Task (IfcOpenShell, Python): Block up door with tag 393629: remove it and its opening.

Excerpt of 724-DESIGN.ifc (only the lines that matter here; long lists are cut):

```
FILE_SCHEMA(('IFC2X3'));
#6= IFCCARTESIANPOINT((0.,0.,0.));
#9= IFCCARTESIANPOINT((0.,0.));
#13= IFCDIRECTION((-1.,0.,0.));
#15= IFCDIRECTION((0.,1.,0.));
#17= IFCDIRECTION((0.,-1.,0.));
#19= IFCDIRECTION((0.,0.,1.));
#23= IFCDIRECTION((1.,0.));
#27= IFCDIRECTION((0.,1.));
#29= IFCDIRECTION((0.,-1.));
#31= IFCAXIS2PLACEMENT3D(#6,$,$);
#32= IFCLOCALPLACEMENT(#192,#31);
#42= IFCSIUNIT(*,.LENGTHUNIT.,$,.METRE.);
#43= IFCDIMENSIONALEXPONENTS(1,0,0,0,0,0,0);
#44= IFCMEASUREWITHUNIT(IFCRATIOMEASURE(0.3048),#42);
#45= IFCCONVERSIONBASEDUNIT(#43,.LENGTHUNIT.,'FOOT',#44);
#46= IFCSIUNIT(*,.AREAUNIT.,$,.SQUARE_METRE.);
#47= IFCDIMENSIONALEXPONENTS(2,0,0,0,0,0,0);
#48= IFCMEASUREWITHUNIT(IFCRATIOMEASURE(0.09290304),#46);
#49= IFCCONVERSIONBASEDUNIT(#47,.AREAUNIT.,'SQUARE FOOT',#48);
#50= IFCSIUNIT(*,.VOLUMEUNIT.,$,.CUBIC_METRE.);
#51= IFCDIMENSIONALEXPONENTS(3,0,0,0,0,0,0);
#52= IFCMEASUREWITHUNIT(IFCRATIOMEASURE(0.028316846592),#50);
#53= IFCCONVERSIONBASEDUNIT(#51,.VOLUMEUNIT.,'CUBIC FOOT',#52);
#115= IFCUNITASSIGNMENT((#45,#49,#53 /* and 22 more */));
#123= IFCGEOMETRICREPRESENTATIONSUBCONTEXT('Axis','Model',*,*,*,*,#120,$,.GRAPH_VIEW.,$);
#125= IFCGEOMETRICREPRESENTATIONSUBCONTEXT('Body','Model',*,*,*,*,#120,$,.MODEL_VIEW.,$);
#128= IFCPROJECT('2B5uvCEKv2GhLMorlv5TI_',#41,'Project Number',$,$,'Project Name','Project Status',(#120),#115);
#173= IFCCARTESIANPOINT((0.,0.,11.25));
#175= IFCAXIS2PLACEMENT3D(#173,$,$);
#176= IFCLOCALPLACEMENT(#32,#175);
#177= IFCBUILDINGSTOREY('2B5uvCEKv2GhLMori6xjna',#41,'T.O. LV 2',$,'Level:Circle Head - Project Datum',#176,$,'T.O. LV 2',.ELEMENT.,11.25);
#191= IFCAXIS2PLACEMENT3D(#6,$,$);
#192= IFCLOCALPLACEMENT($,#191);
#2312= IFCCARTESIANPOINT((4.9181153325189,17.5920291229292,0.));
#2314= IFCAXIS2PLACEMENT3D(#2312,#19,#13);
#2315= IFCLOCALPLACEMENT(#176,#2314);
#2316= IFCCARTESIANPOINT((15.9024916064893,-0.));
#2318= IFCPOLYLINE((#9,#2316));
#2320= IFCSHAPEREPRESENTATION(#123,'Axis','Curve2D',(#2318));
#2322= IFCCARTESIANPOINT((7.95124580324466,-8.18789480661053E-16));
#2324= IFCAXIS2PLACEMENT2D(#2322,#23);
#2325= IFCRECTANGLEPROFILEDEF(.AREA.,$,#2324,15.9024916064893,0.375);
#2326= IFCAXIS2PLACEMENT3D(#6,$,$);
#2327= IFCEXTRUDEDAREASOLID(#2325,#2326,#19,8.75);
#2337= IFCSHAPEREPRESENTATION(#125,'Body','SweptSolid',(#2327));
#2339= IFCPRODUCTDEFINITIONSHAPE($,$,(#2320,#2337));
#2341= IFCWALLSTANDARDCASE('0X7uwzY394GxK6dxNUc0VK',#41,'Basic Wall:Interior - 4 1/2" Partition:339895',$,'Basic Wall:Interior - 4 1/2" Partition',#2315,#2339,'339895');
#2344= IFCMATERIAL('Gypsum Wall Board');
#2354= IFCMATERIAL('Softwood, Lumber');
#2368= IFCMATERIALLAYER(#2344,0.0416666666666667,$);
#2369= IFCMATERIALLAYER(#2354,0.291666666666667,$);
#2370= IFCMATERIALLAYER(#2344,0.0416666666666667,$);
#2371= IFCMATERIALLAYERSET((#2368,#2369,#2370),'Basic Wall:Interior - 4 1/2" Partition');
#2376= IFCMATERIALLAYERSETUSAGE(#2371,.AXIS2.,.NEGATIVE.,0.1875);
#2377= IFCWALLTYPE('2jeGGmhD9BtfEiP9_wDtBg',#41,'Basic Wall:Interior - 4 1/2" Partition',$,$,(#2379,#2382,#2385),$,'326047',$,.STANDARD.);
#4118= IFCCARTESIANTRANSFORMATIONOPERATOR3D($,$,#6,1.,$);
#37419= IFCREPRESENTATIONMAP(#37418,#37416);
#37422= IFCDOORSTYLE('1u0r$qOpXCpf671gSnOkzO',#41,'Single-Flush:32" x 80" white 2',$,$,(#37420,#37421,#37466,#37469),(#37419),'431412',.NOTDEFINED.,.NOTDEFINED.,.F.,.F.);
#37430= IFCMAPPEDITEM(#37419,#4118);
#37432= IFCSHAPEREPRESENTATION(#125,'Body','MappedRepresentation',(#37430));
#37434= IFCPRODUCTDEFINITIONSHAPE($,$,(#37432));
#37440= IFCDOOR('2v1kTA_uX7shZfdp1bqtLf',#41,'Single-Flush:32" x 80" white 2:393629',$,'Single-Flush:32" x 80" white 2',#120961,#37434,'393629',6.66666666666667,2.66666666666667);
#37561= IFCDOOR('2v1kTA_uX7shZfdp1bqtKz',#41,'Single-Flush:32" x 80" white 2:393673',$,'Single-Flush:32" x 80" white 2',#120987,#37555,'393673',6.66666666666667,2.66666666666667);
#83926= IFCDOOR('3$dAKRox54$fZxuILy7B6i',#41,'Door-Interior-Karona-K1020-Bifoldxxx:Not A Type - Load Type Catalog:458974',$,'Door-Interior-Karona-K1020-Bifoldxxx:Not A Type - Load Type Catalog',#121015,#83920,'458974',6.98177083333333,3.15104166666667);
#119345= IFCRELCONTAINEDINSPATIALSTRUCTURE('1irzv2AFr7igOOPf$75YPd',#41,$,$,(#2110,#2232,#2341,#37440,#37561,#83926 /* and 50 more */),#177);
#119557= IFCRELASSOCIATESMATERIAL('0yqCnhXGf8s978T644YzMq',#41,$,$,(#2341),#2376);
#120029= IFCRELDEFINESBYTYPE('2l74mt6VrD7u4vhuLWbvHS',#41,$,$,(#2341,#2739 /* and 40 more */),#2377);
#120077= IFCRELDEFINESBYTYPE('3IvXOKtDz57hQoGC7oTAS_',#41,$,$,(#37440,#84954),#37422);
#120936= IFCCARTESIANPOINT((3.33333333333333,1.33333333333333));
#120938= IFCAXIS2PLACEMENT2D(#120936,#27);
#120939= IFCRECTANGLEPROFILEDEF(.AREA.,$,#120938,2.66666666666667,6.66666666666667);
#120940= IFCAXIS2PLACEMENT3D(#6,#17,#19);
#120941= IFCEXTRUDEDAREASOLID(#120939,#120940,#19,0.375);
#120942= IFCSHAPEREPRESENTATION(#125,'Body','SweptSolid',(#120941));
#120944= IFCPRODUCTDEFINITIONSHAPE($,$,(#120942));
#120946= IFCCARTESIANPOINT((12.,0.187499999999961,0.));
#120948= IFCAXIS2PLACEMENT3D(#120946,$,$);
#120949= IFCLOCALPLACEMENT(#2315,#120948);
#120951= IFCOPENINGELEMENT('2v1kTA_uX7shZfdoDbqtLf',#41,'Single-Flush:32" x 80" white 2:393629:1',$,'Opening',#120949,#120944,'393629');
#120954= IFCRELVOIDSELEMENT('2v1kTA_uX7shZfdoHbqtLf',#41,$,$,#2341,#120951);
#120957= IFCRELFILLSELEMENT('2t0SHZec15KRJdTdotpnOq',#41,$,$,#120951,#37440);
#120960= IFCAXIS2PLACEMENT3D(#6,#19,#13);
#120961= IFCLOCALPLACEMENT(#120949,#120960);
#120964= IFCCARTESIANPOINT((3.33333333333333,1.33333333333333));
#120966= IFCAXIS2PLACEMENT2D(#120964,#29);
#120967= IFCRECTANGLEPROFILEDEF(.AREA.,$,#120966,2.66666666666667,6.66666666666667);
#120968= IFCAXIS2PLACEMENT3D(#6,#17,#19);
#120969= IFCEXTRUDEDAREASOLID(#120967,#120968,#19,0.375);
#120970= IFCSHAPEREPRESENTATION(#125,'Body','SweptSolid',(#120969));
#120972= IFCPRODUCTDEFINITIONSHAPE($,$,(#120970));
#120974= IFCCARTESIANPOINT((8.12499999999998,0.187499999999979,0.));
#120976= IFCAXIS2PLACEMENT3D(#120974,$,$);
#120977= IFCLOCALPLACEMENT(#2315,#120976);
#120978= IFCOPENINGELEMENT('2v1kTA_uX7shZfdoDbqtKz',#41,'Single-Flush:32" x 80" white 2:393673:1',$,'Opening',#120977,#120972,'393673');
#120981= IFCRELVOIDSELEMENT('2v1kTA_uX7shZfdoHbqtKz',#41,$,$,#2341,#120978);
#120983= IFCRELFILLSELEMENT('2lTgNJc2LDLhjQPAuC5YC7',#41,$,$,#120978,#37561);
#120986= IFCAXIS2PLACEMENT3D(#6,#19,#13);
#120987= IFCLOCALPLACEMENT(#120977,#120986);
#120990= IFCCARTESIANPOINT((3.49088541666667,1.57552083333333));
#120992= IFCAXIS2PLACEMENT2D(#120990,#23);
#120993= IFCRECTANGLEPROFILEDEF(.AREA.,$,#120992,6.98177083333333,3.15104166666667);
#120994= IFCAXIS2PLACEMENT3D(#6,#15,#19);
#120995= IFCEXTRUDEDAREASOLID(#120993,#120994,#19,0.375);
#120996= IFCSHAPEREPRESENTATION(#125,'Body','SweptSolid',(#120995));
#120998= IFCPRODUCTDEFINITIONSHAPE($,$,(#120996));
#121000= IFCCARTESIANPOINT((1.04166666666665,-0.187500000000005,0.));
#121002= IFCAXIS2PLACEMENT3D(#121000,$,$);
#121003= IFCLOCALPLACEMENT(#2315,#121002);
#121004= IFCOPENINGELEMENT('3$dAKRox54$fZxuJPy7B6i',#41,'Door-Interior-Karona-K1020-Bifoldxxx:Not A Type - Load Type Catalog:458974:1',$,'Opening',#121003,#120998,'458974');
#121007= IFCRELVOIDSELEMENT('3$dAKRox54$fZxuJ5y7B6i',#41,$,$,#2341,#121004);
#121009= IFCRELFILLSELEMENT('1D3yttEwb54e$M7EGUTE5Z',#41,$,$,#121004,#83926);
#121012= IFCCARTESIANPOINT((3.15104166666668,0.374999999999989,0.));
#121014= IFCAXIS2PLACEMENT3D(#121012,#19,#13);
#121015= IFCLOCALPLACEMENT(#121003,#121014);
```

```python
import ifcopenshell
import ifcopenshell.api.feature
import ifcopenshell.api.root
import ifcopenshell.geom
import ifcopenshell.util.shape

model = ifcopenshell.open("724-DESIGN.ifc")
settings = ifcopenshell.geom.settings()


def volume(element):
    """Net volume in cubic metres, openings subtracted."""
    shape = ifcopenshell.geom.create_shape(settings, element)
    return ifcopenshell.util.shape.get_volume(shape.geometry)


door = model.by_guid("2v1kTA_uX7shZfdp1bqtLf")
opening = door.FillsVoids[0].RelatingOpeningElement
wall = opening.VoidsElements[0].RelatingBuildingElement
before = volume(wall)

ifcopenshell.api.root.remove_product(model, product=door)
ifcopenshell.api.feature.remove_feature(model, feature=opening)

after = volume(wall)

print(f"wall volume {before:.3f} -> {after:.3f} m3")

model.write("724-DESIGN_v2.ifc")
```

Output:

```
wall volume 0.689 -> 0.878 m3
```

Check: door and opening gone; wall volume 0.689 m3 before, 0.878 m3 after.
